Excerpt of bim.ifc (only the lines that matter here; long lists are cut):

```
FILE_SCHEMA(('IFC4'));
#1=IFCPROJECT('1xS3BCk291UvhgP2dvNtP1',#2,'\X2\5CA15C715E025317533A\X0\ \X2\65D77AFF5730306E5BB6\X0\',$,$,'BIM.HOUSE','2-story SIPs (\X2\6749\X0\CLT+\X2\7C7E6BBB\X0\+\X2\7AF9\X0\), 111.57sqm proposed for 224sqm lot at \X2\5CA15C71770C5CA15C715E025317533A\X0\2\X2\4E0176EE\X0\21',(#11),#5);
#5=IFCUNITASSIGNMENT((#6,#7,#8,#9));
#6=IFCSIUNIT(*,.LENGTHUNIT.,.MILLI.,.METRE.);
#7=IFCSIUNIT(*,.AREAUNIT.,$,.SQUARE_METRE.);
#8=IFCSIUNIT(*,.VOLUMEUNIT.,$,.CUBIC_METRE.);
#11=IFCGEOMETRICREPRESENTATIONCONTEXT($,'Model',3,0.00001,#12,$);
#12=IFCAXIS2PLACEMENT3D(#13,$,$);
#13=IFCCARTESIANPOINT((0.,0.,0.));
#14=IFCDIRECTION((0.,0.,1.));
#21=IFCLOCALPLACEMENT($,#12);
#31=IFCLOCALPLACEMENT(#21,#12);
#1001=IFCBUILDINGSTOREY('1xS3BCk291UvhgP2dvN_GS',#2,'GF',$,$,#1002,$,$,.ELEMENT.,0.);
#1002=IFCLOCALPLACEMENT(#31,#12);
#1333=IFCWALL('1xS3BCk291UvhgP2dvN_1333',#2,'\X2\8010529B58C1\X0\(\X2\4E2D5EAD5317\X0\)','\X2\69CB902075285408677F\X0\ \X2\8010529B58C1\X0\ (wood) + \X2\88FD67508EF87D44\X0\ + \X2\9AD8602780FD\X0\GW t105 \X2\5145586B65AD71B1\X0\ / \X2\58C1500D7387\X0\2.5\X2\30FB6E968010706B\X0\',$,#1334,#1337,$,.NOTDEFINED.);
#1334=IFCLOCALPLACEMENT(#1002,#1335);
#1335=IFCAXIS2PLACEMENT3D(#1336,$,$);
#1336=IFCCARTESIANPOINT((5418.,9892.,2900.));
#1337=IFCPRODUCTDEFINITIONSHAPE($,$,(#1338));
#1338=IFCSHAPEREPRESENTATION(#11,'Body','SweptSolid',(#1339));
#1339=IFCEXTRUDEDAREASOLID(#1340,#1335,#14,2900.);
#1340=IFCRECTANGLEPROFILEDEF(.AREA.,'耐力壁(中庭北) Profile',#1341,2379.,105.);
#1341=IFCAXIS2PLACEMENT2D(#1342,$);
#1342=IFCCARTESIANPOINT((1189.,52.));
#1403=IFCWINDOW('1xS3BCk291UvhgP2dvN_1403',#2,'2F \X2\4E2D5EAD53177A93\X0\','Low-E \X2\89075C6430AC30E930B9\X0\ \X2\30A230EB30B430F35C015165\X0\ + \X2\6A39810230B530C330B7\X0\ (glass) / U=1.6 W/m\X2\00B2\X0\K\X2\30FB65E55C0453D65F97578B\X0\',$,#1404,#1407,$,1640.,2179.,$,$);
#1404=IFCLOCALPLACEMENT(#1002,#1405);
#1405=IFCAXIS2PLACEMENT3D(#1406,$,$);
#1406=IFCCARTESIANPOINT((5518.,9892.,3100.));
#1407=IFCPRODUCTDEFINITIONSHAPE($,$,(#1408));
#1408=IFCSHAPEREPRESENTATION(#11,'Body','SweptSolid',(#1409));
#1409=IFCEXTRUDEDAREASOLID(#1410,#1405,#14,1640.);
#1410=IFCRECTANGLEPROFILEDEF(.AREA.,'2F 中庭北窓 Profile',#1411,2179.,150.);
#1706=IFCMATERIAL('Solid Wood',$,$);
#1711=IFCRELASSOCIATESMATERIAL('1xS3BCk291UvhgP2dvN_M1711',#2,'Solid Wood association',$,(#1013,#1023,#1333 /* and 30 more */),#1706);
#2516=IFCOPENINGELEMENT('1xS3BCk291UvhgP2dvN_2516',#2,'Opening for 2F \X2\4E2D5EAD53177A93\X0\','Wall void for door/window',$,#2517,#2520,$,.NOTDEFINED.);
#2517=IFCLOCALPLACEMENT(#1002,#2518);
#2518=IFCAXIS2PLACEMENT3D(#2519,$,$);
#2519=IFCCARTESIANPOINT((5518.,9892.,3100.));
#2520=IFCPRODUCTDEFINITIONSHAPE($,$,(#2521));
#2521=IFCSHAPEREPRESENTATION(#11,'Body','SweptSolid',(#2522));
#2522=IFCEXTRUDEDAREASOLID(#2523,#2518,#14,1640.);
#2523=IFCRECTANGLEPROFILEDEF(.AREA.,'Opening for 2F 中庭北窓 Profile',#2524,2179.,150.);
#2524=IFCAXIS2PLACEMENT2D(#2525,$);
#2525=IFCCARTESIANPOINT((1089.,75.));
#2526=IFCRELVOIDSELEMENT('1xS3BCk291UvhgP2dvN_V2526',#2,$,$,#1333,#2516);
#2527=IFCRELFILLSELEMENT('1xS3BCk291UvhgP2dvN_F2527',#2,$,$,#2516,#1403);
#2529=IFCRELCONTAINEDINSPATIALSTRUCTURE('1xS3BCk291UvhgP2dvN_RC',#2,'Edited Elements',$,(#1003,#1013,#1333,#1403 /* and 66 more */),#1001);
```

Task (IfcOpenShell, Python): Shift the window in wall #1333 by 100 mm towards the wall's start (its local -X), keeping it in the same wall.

```python
import ifcopenshell
import ifcopenshell.api.geometry
import ifcopenshell.util.placement
import ifcopenshell.util.unit

model = ifcopenshell.open("bim.ifc")
unit_scale = ifcopenshell.util.unit.calculate_unit_scale(model)

window = model.by_id(1403)
opening = window.FillsVoids[0].RelatingOpeningElement
wall = opening.VoidsElements[0].RelatingBuildingElement

wall_matrix = ifcopenshell.util.placement.get_local_placement(wall.ObjectPlacement)
shift = wall_matrix[:3, 0] * -0.1 / unit_scale
before = ifcopenshell.util.placement.get_local_placement(window.ObjectPlacement)[:3, 3].copy()

# The window is not placed relative to its opening, so move both.
for product in (opening, window):
    matrix = ifcopenshell.util.placement.get_local_placement(product.ObjectPlacement)
    matrix[:3, 3] += shift
    ifcopenshell.api.geometry.edit_object_placement(model, product=product, matrix=matrix, is_si=False)

after = ifcopenshell.util.placement.get_local_placement(window.ObjectPlacement)[:3, 3]
print("window moved by", (after - before).round(3) + 0.0)

model.write("bim_v2.ifc")
```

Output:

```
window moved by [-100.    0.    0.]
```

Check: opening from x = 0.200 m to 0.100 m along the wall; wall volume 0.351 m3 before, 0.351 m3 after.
